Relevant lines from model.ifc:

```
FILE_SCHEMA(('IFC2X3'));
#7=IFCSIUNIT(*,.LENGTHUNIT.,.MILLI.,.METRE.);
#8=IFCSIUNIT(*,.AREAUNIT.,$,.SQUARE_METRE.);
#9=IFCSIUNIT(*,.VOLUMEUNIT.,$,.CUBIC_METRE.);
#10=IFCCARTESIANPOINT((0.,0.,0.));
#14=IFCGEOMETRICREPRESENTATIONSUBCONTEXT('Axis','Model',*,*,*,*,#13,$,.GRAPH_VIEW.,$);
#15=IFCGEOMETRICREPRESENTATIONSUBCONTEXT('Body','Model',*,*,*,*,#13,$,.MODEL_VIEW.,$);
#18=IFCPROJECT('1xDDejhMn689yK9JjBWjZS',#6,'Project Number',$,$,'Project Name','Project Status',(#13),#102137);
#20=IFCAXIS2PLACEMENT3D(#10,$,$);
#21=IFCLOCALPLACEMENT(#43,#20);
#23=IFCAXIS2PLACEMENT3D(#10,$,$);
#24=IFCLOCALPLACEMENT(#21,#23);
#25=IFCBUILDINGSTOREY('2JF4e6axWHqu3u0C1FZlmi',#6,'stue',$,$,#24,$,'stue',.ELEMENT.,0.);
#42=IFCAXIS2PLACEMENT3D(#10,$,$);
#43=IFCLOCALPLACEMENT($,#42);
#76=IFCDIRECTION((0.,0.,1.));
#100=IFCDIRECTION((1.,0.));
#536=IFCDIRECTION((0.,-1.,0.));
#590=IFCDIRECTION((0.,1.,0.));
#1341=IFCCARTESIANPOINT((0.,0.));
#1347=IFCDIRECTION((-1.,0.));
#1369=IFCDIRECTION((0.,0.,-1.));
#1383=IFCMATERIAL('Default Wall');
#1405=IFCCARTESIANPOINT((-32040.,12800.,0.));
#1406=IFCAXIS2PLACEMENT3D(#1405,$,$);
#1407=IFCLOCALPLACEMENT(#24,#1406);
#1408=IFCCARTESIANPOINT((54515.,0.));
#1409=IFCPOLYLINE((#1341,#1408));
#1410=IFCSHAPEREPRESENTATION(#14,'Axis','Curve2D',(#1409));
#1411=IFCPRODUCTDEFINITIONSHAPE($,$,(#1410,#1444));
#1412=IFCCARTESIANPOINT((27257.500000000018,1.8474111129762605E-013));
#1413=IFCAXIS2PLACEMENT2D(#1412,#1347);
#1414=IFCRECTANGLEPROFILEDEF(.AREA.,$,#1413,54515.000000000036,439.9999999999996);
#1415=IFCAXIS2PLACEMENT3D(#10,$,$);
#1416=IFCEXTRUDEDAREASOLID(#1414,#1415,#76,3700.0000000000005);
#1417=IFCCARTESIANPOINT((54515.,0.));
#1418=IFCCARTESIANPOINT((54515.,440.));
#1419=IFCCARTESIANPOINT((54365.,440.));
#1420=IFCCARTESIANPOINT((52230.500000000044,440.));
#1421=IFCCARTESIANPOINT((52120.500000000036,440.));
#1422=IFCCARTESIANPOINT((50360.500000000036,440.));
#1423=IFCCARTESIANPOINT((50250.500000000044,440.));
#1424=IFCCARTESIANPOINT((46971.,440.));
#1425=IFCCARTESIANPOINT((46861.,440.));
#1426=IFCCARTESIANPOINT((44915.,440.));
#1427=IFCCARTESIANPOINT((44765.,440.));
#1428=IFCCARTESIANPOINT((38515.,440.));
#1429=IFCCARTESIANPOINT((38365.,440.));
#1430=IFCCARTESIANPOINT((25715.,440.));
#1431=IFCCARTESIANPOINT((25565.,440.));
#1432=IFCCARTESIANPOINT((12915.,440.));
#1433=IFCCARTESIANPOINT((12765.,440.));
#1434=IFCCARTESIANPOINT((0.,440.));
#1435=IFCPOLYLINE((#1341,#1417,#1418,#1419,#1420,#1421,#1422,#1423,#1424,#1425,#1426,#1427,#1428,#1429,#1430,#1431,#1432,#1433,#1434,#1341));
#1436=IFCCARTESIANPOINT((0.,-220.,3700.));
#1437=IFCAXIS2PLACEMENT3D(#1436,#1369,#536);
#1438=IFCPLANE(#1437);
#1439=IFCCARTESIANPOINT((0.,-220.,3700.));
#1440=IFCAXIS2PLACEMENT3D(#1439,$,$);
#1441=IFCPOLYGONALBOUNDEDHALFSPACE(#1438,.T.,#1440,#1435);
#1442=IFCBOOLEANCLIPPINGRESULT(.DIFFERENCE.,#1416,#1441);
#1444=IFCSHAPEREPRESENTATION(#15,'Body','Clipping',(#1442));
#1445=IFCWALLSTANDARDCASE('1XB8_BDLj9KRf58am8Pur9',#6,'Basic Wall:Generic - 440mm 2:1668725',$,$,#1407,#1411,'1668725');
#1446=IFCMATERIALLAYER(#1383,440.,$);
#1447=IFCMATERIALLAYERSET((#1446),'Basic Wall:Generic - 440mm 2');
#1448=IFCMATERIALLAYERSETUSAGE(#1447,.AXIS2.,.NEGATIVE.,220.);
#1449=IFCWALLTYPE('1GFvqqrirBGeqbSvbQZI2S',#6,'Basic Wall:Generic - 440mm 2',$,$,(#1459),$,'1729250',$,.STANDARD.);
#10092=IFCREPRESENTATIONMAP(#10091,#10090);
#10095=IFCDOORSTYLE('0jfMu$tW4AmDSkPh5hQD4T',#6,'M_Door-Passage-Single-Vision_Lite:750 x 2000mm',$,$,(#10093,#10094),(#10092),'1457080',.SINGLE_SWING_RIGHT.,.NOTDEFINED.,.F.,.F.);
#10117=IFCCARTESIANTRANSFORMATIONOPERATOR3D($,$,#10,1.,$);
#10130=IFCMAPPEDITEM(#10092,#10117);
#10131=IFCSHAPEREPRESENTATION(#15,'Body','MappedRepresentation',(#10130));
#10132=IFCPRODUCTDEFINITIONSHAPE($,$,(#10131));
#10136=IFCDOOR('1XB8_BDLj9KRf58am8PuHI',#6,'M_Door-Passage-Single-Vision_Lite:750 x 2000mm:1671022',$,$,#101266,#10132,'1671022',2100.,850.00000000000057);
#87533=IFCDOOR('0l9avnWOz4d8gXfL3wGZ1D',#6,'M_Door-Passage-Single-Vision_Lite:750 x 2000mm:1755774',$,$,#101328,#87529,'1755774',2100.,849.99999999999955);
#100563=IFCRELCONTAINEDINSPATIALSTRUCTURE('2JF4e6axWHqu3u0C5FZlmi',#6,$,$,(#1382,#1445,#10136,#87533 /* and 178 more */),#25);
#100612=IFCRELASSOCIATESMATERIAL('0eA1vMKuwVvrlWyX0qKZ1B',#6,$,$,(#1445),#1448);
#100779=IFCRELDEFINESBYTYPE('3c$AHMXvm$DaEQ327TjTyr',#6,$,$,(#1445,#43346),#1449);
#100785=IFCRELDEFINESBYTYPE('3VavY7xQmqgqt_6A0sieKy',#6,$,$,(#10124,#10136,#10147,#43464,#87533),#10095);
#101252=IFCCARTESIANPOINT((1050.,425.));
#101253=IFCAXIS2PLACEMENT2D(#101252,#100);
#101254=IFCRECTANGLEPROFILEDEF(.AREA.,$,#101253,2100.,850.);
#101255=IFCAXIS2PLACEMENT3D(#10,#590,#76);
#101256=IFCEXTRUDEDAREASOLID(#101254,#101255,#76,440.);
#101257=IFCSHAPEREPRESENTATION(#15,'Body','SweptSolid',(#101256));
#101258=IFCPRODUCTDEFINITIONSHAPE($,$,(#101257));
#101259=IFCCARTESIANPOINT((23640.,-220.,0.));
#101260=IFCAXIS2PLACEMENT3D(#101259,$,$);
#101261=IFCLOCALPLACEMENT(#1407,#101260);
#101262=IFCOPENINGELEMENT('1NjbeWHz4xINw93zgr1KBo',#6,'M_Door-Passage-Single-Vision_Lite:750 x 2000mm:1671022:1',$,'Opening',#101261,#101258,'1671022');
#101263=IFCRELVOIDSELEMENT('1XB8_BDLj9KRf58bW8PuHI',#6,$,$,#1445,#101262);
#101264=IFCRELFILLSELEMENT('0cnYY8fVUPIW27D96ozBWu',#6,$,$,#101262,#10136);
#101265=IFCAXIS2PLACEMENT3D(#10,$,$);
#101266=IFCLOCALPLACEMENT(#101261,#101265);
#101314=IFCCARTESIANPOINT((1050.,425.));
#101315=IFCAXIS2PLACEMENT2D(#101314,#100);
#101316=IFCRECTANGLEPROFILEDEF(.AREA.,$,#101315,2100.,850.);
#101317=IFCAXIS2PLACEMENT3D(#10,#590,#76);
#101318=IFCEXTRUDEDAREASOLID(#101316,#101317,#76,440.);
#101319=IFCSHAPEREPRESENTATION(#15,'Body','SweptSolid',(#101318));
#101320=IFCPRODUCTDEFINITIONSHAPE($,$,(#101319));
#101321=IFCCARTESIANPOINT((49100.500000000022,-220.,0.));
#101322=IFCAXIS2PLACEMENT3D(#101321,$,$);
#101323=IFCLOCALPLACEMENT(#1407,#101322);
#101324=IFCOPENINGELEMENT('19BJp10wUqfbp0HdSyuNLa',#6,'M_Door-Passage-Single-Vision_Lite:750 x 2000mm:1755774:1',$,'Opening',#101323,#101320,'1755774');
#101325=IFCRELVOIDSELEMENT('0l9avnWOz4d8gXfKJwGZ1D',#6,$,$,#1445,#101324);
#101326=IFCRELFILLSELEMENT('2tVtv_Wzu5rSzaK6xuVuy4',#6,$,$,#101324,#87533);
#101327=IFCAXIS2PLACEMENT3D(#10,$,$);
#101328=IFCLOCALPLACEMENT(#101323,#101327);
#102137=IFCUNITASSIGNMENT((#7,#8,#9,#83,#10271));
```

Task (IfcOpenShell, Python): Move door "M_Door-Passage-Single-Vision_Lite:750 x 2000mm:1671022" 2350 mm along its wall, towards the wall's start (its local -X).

```python
import ifcopenshell
import ifcopenshell.api.geometry
import ifcopenshell.util.placement
import ifcopenshell.util.unit

model = ifcopenshell.open("model.ifc")
unit_scale = ifcopenshell.util.unit.calculate_unit_scale(model)

door = model.by_id(10136)
opening = door.FillsVoids[0].RelatingOpeningElement
wall = opening.VoidsElements[0].RelatingBuildingElement

wall_matrix = ifcopenshell.util.placement.get_local_placement(wall.ObjectPlacement)
shift = wall_matrix[:3, 0] * -2.35 / unit_scale
before = ifcopenshell.util.placement.get_local_placement(door.ObjectPlacement)[:3, 3].copy()

# The door is placed relative to its opening, so it follows when the opening moves.
matrix = ifcopenshell.util.placement.get_local_placement(opening.ObjectPlacement)
matrix[:3, 3] += shift
ifcopenshell.api.geometry.edit_object_placement(
    model, product=opening, matrix=matrix, is_si=False, should_transform_children=True
)

after = ifcopenshell.util.placement.get_local_placement(door.ObjectPlacement)[:3, 3]
print("door moved by", (after - before).round(3) + 0.0)

model.write("model_rev.ifc")
```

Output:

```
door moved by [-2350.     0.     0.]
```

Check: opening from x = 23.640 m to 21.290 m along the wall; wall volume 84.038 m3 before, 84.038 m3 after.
